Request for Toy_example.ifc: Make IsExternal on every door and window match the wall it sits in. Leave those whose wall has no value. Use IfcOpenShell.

First a look at what the model holds.

```python
import ifcopenshell
import ifcopenshell.util.element

model = ifcopenshell.open("Toy_example.ifc")
print(model.schema)
seen = {}
for e in model.by_type("IfcDoor") + model.by_type("IfcWindow"):
    if not e.FillsVoids:
        continue
    host = e.FillsVoids[0].RelatingOpeningElement.VoidsElements[0].RelatingBuildingElement
    own = ifcopenshell.util.element.get_pset(e, f"Pset_{e.is_a()[3:].removesuffix('StandardCase')}Common", "IsExternal")
    wall = ifcopenshell.util.element.get_pset(host, "Pset_WallCommon", "IsExternal")
    seen[e.is_a(), own, wall] = seen.get((e.is_a(), own, wall), 0) + 1
for (cls, own, wall), count in sorted(seen.items(), key=str):
    print(count, cls, "IsExternal:", own, "| host wall:", wall)
```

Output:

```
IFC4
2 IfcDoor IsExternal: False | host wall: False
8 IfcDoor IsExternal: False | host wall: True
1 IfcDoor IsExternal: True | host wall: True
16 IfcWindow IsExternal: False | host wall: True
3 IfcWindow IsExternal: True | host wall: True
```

```python
import ifcopenshell
import ifcopenshell.api.pset
import ifcopenshell.util.element

model = ifcopenshell.open("Toy_example.ifc")

count = 0
for ifc_class, pset_name in (("IfcDoor", "Pset_DoorCommon"), ("IfcWindow", "Pset_WindowCommon")):
    for e in model.by_type(ifc_class):
        if not e.FillsVoids:
            continue
        host = e.FillsVoids[0].RelatingOpeningElement.VoidsElements[0].RelatingBuildingElement
        external = ifcopenshell.util.element.get_pset(host, "Pset_WallCommon", "IsExternal")
        if external is None or ifcopenshell.util.element.get_pset(e, pset_name, "IsExternal") == external:
            continue
        pset = ifcopenshell.api.pset.add_pset(model, product=e, name=pset_name)
        ifcopenshell.api.pset.edit_pset(model, pset=pset, properties={"IsExternal": external})
        count += 1

print(count, "updated")

model.write("Toy_example_v2.ifc")
```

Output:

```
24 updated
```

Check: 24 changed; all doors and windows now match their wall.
